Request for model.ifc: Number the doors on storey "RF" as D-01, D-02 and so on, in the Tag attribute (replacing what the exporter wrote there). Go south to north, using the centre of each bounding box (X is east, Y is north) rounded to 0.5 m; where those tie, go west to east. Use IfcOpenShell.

First a look at what the model holds.

```python
import ifcopenshell
import ifcopenshell.util.element
import ifcopenshell.util.placement

model = ifcopenshell.open("model.ifc")
print(model.schema)
storey = next(s for s in model.by_type("IfcBuildingStorey") if s.Name == "RF")
doors = [e for e in ifcopenshell.util.element.get_decomposition(storey) if e.is_a("IfcDoor")]
for e in sorted(doors, key=lambda e: e.id()):
    origin = ifcopenshell.util.placement.get_local_placement(e.ObjectPlacement)[:3, 3]
    print(e.id(), e.Tag, e.Name, origin.round(2) + 0.0, sep=" | ")
```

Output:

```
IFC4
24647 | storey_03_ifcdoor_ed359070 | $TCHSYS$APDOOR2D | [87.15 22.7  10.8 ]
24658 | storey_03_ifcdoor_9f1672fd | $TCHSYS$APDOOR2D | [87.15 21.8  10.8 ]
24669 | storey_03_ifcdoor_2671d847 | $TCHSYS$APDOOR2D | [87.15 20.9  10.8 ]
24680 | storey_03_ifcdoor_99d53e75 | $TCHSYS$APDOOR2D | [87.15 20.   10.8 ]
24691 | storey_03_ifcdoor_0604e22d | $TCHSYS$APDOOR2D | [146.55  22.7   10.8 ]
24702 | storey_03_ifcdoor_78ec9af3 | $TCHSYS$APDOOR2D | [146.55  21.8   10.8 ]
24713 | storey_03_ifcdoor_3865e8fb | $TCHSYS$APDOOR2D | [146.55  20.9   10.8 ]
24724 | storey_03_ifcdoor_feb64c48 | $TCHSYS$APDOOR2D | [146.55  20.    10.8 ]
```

```python
import ifcopenshell
import ifcopenshell.geom
import ifcopenshell.util.element
import ifcopenshell.util.shape

model = ifcopenshell.open("model.ifc")
settings = ifcopenshell.geom.settings()
settings.set("use-world-coords", True)


def centre(element):
    shape = ifcopenshell.geom.create_shape(settings, element)
    return ifcopenshell.util.shape.get_bbox_centroid(shape.geometry)


storey = next(s for s in model.by_type("IfcBuildingStorey") if s.Name == "RF")
doors = [e for e in ifcopenshell.util.element.get_decomposition(storey) if e.is_a("IfcDoor")]

# Insertion points can sit at a corner or the storey origin, so sort by the geometry (in metres).
centres = {e: centre(e) for e in doors}
doors.sort(key=lambda e: (round(centres[e][1] / 0.5), centres[e][0]))

for i, e in enumerate(doors, start=1):
    number = f"D-{i:02d}"
    e.Tag = number
    print(e.id(), number)

model.write("model_v2.ifc")
```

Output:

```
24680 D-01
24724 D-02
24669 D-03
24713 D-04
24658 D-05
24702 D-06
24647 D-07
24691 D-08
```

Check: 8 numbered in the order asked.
